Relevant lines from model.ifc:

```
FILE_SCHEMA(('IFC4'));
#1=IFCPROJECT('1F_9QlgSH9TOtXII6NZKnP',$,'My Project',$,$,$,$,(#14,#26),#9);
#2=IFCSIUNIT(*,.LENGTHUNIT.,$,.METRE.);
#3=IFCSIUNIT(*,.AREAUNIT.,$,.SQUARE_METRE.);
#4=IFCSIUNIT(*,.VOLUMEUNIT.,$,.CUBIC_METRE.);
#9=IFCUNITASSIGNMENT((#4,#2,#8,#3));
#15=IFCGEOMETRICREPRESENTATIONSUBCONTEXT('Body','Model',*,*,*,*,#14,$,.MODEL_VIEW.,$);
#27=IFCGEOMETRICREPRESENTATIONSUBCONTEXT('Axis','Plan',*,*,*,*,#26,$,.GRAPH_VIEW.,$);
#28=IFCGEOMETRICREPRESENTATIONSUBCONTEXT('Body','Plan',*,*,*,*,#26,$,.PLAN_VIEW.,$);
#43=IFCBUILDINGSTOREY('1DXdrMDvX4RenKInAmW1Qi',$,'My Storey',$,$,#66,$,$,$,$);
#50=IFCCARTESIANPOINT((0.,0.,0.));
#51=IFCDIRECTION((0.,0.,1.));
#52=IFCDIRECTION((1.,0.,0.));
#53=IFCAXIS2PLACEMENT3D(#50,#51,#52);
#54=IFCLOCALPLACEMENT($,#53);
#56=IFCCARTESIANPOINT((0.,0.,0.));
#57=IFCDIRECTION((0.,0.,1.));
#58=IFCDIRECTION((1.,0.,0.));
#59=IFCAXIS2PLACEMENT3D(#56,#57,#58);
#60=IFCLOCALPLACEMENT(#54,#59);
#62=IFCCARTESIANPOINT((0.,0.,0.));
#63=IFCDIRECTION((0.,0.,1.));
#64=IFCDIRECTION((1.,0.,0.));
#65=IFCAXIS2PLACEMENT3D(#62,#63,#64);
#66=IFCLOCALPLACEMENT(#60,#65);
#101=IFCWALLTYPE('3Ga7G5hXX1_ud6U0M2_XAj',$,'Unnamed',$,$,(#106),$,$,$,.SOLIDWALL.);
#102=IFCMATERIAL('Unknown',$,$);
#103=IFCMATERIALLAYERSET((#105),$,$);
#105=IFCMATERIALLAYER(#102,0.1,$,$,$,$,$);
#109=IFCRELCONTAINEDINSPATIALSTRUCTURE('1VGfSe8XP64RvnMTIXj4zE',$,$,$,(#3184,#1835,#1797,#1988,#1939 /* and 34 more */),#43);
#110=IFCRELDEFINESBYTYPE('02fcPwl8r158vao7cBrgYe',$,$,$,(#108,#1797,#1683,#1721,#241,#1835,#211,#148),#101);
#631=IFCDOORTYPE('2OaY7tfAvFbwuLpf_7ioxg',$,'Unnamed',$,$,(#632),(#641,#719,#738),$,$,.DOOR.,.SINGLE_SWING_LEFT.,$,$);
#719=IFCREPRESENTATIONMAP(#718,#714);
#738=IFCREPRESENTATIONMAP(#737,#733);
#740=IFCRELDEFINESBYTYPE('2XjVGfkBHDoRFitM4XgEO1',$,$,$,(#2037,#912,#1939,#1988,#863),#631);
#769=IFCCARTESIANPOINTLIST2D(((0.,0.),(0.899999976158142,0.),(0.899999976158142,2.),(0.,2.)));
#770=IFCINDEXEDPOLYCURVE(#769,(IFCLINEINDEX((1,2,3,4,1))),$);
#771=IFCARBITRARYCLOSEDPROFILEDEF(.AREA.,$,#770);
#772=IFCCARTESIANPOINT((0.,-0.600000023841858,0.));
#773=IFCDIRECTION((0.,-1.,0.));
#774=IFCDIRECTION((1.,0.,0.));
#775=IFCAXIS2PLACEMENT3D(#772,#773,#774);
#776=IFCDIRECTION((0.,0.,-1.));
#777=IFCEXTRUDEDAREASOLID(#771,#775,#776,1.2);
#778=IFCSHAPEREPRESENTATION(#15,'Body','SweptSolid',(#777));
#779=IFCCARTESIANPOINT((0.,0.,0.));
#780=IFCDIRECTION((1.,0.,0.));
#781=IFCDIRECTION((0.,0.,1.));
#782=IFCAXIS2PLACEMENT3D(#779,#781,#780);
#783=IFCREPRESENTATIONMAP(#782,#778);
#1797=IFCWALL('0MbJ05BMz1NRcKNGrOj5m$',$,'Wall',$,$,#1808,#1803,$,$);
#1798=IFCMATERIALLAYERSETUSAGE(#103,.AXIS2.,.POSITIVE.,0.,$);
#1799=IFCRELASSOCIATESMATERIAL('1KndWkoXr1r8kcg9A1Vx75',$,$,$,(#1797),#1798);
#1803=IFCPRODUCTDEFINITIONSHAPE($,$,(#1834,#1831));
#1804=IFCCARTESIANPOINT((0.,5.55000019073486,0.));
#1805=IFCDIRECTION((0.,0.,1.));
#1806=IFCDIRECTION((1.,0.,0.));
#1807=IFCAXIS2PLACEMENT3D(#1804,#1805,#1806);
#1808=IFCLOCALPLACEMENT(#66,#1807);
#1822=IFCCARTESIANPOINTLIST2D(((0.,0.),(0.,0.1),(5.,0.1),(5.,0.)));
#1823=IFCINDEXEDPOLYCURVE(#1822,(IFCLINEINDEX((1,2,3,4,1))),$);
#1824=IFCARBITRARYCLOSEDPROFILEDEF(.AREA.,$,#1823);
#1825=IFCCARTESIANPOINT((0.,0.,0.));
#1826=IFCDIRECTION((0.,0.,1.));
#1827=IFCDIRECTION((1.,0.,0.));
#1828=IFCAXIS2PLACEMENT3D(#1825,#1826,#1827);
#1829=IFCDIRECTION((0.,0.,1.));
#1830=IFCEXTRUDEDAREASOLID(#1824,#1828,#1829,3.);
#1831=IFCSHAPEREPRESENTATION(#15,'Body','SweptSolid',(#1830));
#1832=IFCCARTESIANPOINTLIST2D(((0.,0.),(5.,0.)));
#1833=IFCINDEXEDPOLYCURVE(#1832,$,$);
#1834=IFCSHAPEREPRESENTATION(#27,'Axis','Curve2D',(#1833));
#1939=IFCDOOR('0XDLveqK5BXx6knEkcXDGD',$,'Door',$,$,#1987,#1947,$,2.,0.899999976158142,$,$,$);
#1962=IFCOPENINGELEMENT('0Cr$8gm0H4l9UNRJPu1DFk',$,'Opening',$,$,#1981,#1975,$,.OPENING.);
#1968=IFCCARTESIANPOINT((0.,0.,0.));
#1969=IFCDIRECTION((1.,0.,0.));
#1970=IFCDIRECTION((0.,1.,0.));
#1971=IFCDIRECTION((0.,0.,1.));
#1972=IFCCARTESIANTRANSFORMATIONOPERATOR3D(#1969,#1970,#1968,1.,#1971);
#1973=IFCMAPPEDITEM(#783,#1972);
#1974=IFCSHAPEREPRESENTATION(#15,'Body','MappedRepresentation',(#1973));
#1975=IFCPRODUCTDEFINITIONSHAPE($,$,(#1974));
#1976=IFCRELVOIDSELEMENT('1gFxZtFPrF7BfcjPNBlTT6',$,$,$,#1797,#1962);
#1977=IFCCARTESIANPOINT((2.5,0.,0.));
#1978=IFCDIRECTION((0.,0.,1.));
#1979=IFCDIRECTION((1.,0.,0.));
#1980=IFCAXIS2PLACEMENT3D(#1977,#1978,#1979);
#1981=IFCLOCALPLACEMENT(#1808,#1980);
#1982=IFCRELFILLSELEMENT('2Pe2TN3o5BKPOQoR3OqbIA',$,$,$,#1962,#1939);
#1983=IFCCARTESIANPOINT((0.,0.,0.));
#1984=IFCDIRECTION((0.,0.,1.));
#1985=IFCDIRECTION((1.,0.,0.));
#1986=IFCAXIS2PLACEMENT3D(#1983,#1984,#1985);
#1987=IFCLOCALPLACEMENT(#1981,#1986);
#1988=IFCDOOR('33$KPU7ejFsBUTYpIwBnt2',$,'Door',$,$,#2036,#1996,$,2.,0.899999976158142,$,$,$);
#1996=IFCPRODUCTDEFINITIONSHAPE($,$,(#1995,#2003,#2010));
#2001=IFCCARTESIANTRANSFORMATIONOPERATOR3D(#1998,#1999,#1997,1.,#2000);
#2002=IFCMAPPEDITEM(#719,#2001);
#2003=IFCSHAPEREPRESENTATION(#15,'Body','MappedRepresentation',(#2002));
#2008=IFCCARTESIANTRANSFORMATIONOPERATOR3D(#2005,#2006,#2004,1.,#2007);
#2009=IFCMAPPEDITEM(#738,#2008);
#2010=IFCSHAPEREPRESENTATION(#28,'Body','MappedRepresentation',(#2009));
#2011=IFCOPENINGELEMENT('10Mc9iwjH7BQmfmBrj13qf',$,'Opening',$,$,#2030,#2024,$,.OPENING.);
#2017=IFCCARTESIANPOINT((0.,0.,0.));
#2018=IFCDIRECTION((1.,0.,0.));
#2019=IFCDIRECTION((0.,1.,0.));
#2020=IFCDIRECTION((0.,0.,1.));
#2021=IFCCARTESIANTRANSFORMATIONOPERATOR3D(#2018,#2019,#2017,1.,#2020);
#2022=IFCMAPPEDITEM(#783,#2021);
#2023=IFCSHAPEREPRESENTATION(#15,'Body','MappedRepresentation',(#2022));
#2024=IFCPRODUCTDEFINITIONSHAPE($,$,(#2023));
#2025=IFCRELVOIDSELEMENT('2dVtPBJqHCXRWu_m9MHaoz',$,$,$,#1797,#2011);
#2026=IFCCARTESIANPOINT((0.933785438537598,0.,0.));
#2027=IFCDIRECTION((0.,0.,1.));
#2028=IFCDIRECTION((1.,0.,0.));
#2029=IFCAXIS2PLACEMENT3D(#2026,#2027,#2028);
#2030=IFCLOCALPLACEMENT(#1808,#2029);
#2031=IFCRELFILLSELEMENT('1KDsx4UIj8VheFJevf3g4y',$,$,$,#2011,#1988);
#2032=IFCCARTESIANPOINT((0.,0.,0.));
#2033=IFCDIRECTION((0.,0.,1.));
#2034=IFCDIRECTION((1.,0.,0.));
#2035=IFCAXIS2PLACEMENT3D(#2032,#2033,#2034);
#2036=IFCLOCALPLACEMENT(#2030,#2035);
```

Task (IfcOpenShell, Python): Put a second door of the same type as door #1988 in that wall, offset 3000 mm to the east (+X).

```python
import ifcopenshell
import ifcopenshell.api.feature
import ifcopenshell.api.geometry
import ifcopenshell.api.root
import ifcopenshell.geom
import ifcopenshell.util.element
import ifcopenshell.util.placement
import ifcopenshell.util.shape

model = ifcopenshell.open("model.ifc")
settings = ifcopenshell.geom.settings()


def volume(element):
    """Net volume in cubic metres, openings subtracted."""
    shape = ifcopenshell.geom.create_shape(settings, element)
    return ifcopenshell.util.shape.get_volume(shape.geometry)


door = model.by_guid("33$KPU7ejFsBUTYpIwBnt2")
opening = door.FillsVoids[0].RelatingOpeningElement
wall = opening.VoidsElements[0].RelatingBuildingElement
before = volume(wall)
shift = ifcopenshell.util.placement.get_local_placement(wall.ObjectPlacement)[:3, 0] * 3.0

# copy_class copies the void relationship, type, container and properties, but no geometry.
new_opening = ifcopenshell.api.root.copy_class(model, product=opening)
new_opening.Representation = ifcopenshell.util.element.copy_deep(
    model, opening.Representation, exclude=["IfcGeometricRepresentationContext", "IfcRepresentationMap"]
)
new_door = ifcopenshell.api.root.copy_class(model, product=door)
new_door.Representation = ifcopenshell.util.element.copy_deep(
    model, door.Representation, exclude=["IfcGeometricRepresentationContext", "IfcRepresentationMap"]
)
ifcopenshell.api.feature.add_filling(model, opening=new_opening, element=new_door)

for old, new in ((opening, new_opening), (door, new_door)):
    matrix = ifcopenshell.util.placement.get_local_placement(old.ObjectPlacement)
    matrix[:3, 3] += shift
    ifcopenshell.api.geometry.edit_object_placement(model, product=new, matrix=matrix, is_si=False)

after = volume(wall)

print(f"wall volume {before:.3f} -> {after:.3f} m3")

model.write("model_updated.ifc")
```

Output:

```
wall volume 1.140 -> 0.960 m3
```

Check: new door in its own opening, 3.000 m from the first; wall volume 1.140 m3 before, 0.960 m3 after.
